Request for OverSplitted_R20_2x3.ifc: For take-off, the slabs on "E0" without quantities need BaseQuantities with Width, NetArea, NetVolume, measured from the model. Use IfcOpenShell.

First a look at what the model holds.

```python
import ifcopenshell
import ifcopenshell.util.element
import ifcopenshell.util.unit

model = ifcopenshell.open("OverSplitted_R20_2x3.ifc")
print(model.schema)
for unit_type in ("LENGTHUNIT", "AREAUNIT", "VOLUMEUNIT"):
    print(unit_type, ifcopenshell.util.unit.calculate_unit_scale(model, unit_type))
storey = next(s for s in model.by_type("IfcBuildingStorey") if s.Name == "E0")
slabs = [e for e in ifcopenshell.util.element.get_decomposition(storey) if e.is_a("IfcSlab")]
for e in sorted(slabs, key=lambda e: e.id()):
    print(e.id(), e.is_a(), e.Name, list(ifcopenshell.util.element.get_psets(e, qtos_only=True)), sep=" | ")
```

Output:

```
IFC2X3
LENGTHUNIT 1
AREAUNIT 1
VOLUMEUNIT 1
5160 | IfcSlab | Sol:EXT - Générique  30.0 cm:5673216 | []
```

```python
import ifcopenshell
import ifcopenshell.api.pset
import ifcopenshell.geom
import ifcopenshell.util.element
import ifcopenshell.util.shape
import ifcopenshell.util.unit

model = ifcopenshell.open("OverSplitted_R20_2x3.ifc")
unit_scale = ifcopenshell.util.unit.calculate_unit_scale(model)
area_scale = ifcopenshell.util.unit.calculate_unit_scale(model, "AREAUNIT")
volume_scale = ifcopenshell.util.unit.calculate_unit_scale(model, "VOLUMEUNIT")
settings = ifcopenshell.geom.settings()

storey = next(s for s in model.by_type("IfcBuildingStorey") if s.Name == "E0")
slabs = [e for e in ifcopenshell.util.element.get_decomposition(storey) if e.is_a("IfcSlab")]

for e in sorted(slabs, key=lambda e: e.id()):
    if ifcopenshell.util.element.get_psets(e, qtos_only=True, should_inherit=False):
        continue
    # Geometry comes back in metres, in the element's own axes.
    shape = ifcopenshell.geom.create_shape(settings, e)
    values = {
        "Width": ifcopenshell.util.shape.get_z(shape.geometry) / unit_scale,
        "NetArea": ifcopenshell.util.shape.get_footprint_area(shape.geometry) / area_scale,
        "NetVolume": ifcopenshell.util.shape.get_volume(shape.geometry) / volume_scale,
    }
    qto = ifcopenshell.api.pset.add_qto(model, product=e, name="BaseQuantities")
    ifcopenshell.api.pset.edit_qto(model, qto=qto, properties=values)
    print(e.id(), {k: round(v, 3) for k, v in values.items()})

model.write("OverSplitted_R20_2x3_updated.ifc")
```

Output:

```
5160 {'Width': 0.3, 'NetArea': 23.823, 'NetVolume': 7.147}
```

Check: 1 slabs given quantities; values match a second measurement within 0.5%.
